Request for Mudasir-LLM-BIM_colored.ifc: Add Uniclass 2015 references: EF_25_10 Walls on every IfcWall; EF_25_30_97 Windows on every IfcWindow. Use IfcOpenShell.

First a look at what the model holds.

```python
import ifcopenshell

model = ifcopenshell.open("Mudasir-LLM-BIM_colored.ifc")
print(model.schema)
print("classifications:", [c.Name for c in model.by_type("IfcClassification")])
for ifc_class in ("IfcDoor", "IfcRoof", "IfcStair", "IfcWall", "IfcWindow"):
    print(ifc_class, len(model.by_type(ifc_class)))
```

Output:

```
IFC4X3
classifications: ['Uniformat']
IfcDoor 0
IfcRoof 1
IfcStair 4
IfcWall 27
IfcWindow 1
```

```python
import ifcopenshell
import ifcopenshell.api.classification

model = ifcopenshell.open("Mudasir-LLM-BIM_colored.ifc")

system = ifcopenshell.api.classification.add_classification(model, classification="Uniclass 2015")

codes = {
    "IfcWall": ("EF_25_10", "Walls"),
    "IfcWindow": ("EF_25_30_97", "Windows"),
}
for ifc_class, (code, name) in codes.items():
    products = model.by_type(ifc_class)
    ifcopenshell.api.classification.add_reference(
        model, products=products, classification=system, identification=code, name=name
    )
    print(code, len(products))

model.write("Mudasir-LLM-BIM_colored_updated.ifc")
```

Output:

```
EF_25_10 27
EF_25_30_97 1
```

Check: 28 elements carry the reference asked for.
